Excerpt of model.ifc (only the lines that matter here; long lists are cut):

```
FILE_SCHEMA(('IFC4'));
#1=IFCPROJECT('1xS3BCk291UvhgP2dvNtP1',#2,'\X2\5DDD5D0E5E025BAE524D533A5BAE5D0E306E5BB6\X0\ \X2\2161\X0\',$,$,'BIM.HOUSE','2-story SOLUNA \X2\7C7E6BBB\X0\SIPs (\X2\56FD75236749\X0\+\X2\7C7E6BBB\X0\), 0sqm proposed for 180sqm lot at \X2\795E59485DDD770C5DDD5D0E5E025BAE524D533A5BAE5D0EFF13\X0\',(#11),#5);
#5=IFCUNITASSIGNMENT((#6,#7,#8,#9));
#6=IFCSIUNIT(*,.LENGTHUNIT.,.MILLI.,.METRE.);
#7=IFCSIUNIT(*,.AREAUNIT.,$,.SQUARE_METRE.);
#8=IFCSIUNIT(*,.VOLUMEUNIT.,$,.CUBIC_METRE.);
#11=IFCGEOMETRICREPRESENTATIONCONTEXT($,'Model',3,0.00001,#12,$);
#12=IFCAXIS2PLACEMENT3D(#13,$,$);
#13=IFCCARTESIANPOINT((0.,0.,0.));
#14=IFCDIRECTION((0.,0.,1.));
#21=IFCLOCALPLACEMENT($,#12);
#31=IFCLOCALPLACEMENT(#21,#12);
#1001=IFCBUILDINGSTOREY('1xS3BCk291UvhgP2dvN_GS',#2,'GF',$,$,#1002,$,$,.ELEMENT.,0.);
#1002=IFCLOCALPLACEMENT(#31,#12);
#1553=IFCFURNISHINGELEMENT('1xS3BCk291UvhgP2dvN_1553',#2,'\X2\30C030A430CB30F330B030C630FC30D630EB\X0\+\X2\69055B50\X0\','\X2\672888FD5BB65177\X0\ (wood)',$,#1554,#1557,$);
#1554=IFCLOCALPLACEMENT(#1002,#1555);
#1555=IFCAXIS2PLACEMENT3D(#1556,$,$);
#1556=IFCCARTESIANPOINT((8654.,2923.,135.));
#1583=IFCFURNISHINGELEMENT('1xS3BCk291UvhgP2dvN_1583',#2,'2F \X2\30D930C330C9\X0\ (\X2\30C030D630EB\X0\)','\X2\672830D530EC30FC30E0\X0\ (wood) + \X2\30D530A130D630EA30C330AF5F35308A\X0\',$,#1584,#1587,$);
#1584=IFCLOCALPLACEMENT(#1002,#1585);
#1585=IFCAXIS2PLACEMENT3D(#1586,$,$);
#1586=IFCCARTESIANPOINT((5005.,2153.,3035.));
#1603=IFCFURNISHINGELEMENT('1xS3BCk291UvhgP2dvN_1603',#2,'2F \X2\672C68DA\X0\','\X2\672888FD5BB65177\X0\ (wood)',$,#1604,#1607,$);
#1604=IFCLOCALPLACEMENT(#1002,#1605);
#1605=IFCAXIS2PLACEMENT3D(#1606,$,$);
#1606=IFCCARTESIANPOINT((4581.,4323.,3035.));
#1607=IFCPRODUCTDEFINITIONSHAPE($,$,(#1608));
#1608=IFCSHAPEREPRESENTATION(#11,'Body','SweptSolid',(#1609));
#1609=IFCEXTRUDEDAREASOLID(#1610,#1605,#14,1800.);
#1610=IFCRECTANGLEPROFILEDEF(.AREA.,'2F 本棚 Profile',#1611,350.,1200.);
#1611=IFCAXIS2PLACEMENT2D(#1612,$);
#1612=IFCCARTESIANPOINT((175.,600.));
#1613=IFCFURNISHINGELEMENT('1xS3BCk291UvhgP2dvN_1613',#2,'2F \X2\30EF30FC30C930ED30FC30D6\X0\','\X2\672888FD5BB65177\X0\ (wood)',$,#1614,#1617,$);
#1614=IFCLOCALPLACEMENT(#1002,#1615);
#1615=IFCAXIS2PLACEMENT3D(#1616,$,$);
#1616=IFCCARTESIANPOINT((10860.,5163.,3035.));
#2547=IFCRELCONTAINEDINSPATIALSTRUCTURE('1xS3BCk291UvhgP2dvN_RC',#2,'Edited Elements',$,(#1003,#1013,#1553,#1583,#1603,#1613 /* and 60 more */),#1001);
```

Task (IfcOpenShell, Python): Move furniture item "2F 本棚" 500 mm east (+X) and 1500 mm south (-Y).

```python
import ifcopenshell
import ifcopenshell.api.geometry
import ifcopenshell.util.placement

model = ifcopenshell.open("model.ifc")

item = model.by_guid("1xS3BCk291UvhgP2dvN_1603")
matrix = ifcopenshell.util.placement.get_local_placement(item.ObjectPlacement)
matrix[0, 3] += 500.0
matrix[1, 3] -= 1500.0
ifcopenshell.api.geometry.edit_object_placement(model, product=item, matrix=matrix, is_si=False)

print(ifcopenshell.util.placement.get_local_placement(item.ObjectPlacement).round(3) + 0.0)

model.write("model_rev.ifc")
```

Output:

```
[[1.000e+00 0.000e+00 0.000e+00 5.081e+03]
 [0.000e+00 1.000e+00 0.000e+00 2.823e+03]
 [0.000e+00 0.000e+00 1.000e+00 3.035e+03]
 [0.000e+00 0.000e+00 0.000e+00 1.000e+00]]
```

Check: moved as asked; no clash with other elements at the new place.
